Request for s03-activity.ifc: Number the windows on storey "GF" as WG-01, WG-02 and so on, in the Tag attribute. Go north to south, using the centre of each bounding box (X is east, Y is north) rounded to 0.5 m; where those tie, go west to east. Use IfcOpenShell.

First a look at what the model holds.

```python
import ifcopenshell
import ifcopenshell.util.element
import ifcopenshell.util.placement

model = ifcopenshell.open("s03-activity.ifc")
print(model.schema)
storey = next(s for s in model.by_type("IfcBuildingStorey") if s.Name == "GF")
windows = [e for e in ifcopenshell.util.element.get_decomposition(storey) if e.is_a("IfcWindow")]
for e in sorted(windows, key=lambda e: e.id()):
    origin = ifcopenshell.util.placement.get_local_placement(e.ObjectPlacement)[:3, 3]
    print(e.id(), e.Tag, e.Name, origin.round(2) + 0.0, sep=" | ")
```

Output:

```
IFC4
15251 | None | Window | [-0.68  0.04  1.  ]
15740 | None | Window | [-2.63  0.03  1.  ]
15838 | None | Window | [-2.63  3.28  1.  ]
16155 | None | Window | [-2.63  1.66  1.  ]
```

```python
import ifcopenshell
import ifcopenshell.geom
import ifcopenshell.util.element
import ifcopenshell.util.shape

model = ifcopenshell.open("s03-activity.ifc")
settings = ifcopenshell.geom.settings()
settings.set("use-world-coords", True)


def centre(element):
    shape = ifcopenshell.geom.create_shape(settings, element)
    return ifcopenshell.util.shape.get_bbox_centroid(shape.geometry)


storey = next(s for s in model.by_type("IfcBuildingStorey") if s.Name == "GF")
windows = [e for e in ifcopenshell.util.element.get_decomposition(storey) if e.is_a("IfcWindow")]

# Insertion points can sit at a corner or the storey origin, so sort by the geometry (in metres).
centres = {e: centre(e) for e in windows}
windows.sort(key=lambda e: (-round(centres[e][1] / 0.5), centres[e][0]))

for i, e in enumerate(windows, start=1):
    number = f"WG-{i:02d}"
    e.Tag = number
    print(e.id(), number)

model.write("s03-activity_rev.ifc")
```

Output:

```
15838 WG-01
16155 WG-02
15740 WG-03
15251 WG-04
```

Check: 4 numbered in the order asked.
